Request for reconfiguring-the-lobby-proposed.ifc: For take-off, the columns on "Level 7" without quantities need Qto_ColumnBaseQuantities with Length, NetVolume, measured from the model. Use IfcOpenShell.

First a look at what the model holds.

```python
import ifcopenshell
import ifcopenshell.util.element
import ifcopenshell.util.unit

model = ifcopenshell.open("reconfiguring-the-lobby-proposed.ifc")
print(model.schema)
for unit_type in ("LENGTHUNIT", "AREAUNIT", "VOLUMEUNIT"):
    print(unit_type, ifcopenshell.util.unit.calculate_unit_scale(model, unit_type))
storey = next(s for s in model.by_type("IfcBuildingStorey") if s.Name == "Level 7")
columns = [e for e in ifcopenshell.util.element.get_decomposition(storey) if e.is_a("IfcColumn")]
for e in sorted(columns, key=lambda e: e.id()):
    print(e.id(), e.is_a(), e.Name, list(ifcopenshell.util.element.get_psets(e, qtos_only=True)), sep=" | ")
```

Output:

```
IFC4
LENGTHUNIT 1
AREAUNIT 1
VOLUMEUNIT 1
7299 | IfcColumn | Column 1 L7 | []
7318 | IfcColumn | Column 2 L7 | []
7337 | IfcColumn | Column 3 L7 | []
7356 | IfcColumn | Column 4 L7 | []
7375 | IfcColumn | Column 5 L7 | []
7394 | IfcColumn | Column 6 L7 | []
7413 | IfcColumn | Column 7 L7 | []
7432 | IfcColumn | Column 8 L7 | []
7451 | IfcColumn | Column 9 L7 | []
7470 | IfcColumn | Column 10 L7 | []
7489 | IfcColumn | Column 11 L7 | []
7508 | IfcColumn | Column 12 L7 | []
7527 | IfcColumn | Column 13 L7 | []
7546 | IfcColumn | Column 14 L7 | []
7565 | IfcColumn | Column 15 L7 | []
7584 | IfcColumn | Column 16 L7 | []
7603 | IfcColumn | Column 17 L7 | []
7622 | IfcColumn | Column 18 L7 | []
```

```python
import ifcopenshell
import ifcopenshell.api.pset
import ifcopenshell.geom
import ifcopenshell.util.element
import ifcopenshell.util.shape
import ifcopenshell.util.unit

model = ifcopenshell.open("reconfiguring-the-lobby-proposed.ifc")
unit_scale = ifcopenshell.util.unit.calculate_unit_scale(model)
volume_scale = ifcopenshell.util.unit.calculate_unit_scale(model, "VOLUMEUNIT")
settings = ifcopenshell.geom.settings()

storey = next(s for s in model.by_type("IfcBuildingStorey") if s.Name == "Level 7")
columns = [e for e in ifcopenshell.util.element.get_decomposition(storey) if e.is_a("IfcColumn")]

for e in sorted(columns, key=lambda e: e.id()):
    if ifcopenshell.util.element.get_psets(e, qtos_only=True, should_inherit=False):
        continue
    # Geometry comes back in metres, in the element's own axes.
    shape = ifcopenshell.geom.create_shape(settings, e)
    values = {
        "Length": ifcopenshell.util.shape.get_z(shape.geometry) / unit_scale,
        "NetVolume": ifcopenshell.util.shape.get_volume(shape.geometry) / volume_scale,
    }
    qto = ifcopenshell.api.pset.add_qto(model, product=e, name="Qto_ColumnBaseQuantities")
    ifcopenshell.api.pset.edit_qto(model, qto=qto, properties=values)
    print(e.id(), {k: round(v, 3) for k, v in values.items()})

model.write("reconfiguring-the-lobby-proposed_updated.ifc")
```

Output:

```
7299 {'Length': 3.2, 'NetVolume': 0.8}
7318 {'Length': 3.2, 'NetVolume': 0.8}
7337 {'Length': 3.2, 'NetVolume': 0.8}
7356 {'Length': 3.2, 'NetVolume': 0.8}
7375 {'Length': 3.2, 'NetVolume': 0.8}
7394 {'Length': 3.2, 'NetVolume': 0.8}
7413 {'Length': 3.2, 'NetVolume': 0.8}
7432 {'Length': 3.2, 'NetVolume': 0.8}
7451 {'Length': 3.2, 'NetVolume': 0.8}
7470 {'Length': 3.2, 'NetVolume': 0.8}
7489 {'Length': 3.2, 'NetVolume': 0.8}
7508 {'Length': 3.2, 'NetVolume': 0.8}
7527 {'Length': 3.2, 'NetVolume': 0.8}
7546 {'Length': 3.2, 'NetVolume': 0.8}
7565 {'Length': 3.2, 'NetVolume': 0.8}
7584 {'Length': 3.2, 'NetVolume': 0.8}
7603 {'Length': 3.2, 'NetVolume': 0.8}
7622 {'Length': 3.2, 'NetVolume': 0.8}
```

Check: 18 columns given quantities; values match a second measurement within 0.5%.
